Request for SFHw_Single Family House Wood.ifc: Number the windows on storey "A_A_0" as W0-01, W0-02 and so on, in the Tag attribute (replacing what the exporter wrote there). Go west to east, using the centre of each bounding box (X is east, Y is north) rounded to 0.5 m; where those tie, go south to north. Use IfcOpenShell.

First a look at what the model holds.

```python
import ifcopenshell
import ifcopenshell.util.element
import ifcopenshell.util.placement

model = ifcopenshell.open("SFHw_Single Family House Wood.ifc")
print(model.schema)
storey = next(s for s in model.by_type("IfcBuildingStorey") if s.Name == "A_A_0")
windows = [e for e in ifcopenshell.util.element.get_decomposition(storey) if e.is_a("IfcWindow")]
for e in sorted(windows, key=lambda e: e.id()):
    origin = ifcopenshell.util.placement.get_local_placement(e.ObjectPlacement)[:3, 3]
    print(e.id(), e.Tag, e.Name, origin.round(2) + 0.0, sep=" | ")
```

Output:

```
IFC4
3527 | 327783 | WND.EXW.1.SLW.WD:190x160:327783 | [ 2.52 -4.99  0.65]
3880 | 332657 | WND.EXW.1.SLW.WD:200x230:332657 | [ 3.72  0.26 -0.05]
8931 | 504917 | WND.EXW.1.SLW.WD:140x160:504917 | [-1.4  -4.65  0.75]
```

```python
import ifcopenshell
import ifcopenshell.geom
import ifcopenshell.util.element
import ifcopenshell.util.shape

model = ifcopenshell.open("SFHw_Single Family House Wood.ifc")
settings = ifcopenshell.geom.settings()
settings.set("use-world-coords", True)


def centre(element):
    shape = ifcopenshell.geom.create_shape(settings, element)
    return ifcopenshell.util.shape.get_bbox_centroid(shape.geometry)


storey = next(s for s in model.by_type("IfcBuildingStorey") if s.Name == "A_A_0")
windows = [e for e in ifcopenshell.util.element.get_decomposition(storey) if e.is_a("IfcWindow")]

# Insertion points can sit at a corner or the storey origin, so sort by the geometry (in metres).
centres = {e: centre(e) for e in windows}
windows.sort(key=lambda e: (round(centres[e][0] / 0.5), centres[e][1]))

for i, e in enumerate(windows, start=1):
    number = f"W0-{i:02d}"
    e.Tag = number
    print(e.id(), number)

model.write("SFHw_Single Family House Wood-out.ifc")
```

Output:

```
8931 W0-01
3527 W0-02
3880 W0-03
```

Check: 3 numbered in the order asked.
